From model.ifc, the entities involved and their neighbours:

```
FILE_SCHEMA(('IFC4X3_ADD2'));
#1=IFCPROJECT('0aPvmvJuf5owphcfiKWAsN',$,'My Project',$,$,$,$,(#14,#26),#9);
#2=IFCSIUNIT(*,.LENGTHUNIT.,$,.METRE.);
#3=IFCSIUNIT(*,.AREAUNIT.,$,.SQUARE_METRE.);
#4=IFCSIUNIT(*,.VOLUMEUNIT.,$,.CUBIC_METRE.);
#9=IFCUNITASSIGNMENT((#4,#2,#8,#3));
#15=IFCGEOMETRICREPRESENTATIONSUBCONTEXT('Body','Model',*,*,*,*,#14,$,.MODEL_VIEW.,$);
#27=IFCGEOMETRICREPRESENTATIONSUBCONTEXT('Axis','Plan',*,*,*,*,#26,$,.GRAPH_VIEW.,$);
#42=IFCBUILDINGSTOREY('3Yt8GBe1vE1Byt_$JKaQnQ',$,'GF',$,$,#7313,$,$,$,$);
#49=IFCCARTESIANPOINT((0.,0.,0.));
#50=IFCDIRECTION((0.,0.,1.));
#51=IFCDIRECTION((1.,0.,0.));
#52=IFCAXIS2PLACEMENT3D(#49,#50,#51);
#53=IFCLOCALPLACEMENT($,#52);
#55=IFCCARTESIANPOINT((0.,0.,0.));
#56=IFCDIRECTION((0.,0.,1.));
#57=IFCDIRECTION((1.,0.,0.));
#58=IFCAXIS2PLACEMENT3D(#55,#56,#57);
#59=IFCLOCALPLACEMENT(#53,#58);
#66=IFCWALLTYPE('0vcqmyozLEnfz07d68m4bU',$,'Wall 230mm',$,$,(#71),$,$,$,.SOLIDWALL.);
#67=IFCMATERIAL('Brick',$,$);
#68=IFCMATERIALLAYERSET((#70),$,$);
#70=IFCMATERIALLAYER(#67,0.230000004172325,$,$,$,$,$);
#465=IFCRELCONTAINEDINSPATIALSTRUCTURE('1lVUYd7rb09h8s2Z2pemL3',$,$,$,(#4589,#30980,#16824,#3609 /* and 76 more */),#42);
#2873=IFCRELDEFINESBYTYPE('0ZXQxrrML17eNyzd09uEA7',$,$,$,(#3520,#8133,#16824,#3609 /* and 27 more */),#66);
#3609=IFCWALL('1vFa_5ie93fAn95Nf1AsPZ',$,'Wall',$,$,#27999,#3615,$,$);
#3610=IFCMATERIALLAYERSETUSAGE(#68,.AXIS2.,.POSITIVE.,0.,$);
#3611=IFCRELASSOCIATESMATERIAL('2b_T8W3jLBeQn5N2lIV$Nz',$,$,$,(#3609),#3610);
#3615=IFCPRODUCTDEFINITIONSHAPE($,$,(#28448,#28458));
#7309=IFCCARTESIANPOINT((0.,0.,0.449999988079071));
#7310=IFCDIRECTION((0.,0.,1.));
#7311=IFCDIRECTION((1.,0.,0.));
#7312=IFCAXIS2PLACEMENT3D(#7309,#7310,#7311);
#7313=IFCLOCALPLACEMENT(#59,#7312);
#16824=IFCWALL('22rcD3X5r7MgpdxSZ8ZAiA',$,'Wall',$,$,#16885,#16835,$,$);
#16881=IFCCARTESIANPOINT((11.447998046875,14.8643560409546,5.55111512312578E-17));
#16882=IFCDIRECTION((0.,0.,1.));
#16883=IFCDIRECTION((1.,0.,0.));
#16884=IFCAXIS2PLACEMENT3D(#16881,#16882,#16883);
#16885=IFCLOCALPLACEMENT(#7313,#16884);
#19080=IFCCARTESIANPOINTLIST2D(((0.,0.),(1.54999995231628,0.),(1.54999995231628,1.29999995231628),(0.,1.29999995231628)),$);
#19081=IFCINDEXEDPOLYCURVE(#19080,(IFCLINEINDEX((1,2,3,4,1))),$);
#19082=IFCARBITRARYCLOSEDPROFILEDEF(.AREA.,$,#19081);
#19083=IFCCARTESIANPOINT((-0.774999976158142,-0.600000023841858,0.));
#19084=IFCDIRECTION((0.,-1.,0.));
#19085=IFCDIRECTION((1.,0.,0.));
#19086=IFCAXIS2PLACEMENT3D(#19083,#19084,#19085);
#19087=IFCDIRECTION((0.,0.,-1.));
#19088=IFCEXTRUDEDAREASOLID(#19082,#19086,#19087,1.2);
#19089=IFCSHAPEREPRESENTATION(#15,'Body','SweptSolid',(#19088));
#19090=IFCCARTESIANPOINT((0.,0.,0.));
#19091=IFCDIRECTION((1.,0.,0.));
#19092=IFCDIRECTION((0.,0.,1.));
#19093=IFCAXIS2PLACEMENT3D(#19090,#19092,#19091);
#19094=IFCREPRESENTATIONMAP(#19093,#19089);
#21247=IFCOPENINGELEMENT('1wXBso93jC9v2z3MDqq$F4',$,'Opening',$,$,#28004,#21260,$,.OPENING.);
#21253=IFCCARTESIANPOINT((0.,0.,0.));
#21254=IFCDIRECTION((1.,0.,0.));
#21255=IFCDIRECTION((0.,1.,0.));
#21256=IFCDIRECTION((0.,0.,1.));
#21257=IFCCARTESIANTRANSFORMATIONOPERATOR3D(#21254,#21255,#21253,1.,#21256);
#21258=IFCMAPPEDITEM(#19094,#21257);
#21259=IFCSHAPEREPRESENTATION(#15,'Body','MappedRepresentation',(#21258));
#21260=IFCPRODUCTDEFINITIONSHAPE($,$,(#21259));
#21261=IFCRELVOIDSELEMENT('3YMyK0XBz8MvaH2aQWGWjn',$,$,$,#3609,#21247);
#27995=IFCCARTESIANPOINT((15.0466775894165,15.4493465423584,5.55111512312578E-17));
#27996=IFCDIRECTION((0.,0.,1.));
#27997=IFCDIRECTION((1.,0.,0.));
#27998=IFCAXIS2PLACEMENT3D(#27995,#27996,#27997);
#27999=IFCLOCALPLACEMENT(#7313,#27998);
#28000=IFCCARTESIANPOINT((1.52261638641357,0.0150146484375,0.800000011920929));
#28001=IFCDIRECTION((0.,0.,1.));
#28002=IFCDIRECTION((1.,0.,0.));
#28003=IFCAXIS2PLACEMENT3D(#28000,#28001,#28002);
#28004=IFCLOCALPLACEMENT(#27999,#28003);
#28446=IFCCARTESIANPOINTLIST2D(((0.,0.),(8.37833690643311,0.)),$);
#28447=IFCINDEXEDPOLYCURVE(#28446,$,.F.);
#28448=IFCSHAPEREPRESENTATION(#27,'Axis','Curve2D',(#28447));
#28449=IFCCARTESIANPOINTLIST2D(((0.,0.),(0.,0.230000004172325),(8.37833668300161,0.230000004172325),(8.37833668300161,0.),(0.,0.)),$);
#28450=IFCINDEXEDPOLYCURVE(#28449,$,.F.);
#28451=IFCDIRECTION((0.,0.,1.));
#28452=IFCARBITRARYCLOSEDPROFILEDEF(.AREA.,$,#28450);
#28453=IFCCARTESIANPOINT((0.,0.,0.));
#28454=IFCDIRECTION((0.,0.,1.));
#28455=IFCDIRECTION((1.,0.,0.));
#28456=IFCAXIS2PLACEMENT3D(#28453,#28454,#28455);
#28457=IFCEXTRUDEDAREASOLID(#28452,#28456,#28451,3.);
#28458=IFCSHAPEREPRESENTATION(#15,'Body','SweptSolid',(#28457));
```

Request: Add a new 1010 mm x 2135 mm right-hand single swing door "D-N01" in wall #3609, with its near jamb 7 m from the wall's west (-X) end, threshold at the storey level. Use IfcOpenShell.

```python
import numpy as np
import ifcopenshell
import ifcopenshell.api.feature
import ifcopenshell.api.geometry
import ifcopenshell.api.root
import ifcopenshell.api.spatial
import ifcopenshell.geom
import ifcopenshell.util.element
import ifcopenshell.util.placement
import ifcopenshell.util.representation
import ifcopenshell.util.shape
import ifcopenshell.util.unit

model = ifcopenshell.open("model.ifc")
unit_scale = ifcopenshell.util.unit.calculate_unit_scale(model)
settings = ifcopenshell.geom.settings()


def volume(element):
    """Net volume in cubic metres, openings subtracted."""
    shape = ifcopenshell.geom.create_shape(settings, element)
    return ifcopenshell.util.shape.get_volume(shape.geometry)


wall = model.by_guid("1vFa_5ie93fAn95Nf1AsPZ")
storey = ifcopenshell.util.element.get_container(wall, ifc_class="IfcBuildingStorey")
context = ifcopenshell.util.representation.get_context(model, "Model", "Body", "MODEL_VIEW")
before = volume(wall)

width, height, from_end, sill = 1.01, 2.135, 7, 0.0  # metres

# The wall runs along its own X axis, and the end named is its -X end.
wall_shape = ifcopenshell.geom.create_shape(settings, wall)
x, y, z = ifcopenshell.util.shape.get_vertices(wall_shape.geometry).T
start = x.min() + from_end
face, thickness = float(y.min()), float(y.max() - y.min())
wall_matrix = ifcopenshell.util.placement.get_local_placement(wall.ObjectPlacement)
level = ifcopenshell.util.placement.get_local_placement(storey.ObjectPlacement)[2, 3]


def in_wall(x, y):
    """Placement at x, y metres in the wall's axes, at sill height."""
    matrix = wall_matrix.copy()
    matrix[:, 3] = wall_matrix @ np.array([x / unit_scale, y / unit_scale, 0.0, 1.0])
    matrix[2, 3] = level + sill / unit_scale
    return matrix


# Opening: a box that overshoots both wall faces by 50 mm.
opening = ifcopenshell.api.root.create_entity(model, ifc_class="IfcOpeningElement", predefined_type="OPENING")
box = ifcopenshell.api.geometry.add_wall_representation(
    model, context=context, length=width, height=height, thickness=thickness + 0.1
)
ifcopenshell.api.geometry.assign_representation(model, product=opening, representation=box)
ifcopenshell.api.geometry.edit_object_placement(model, product=opening, matrix=in_wall(start, face - 0.05), is_si=False)
ifcopenshell.api.feature.add_feature(model, feature=opening, element=wall)

door = ifcopenshell.api.root.create_entity(model, ifc_class="IfcDoor", name="D-N01", predefined_type="DOOR")
door.OverallWidth, door.OverallHeight = width / unit_scale, height / unit_scale
door.OperationType = "SINGLE_SWING_RIGHT"
body = ifcopenshell.api.geometry.add_door_representation(
    model,
    context=context,
    overall_width=door.OverallWidth,
    overall_height=door.OverallHeight,
    operation_type="SINGLE_SWING_RIGHT",
    lining_properties={"LiningDepth": thickness / unit_scale, "ThresholdDepth": thickness / unit_scale},
)
ifcopenshell.api.geometry.assign_representation(model, product=door, representation=body)
ifcopenshell.api.spatial.assign_container(model, products=[door], relating_structure=storey)
ifcopenshell.api.feature.add_filling(model, opening=opening, element=door)

# The lining spans the wall, so the door starts at the wall face.
ifcopenshell.api.geometry.edit_object_placement(model, product=door, matrix=in_wall(start, face), is_si=False)

after = volume(wall)

print(f"wall volume {before:.3f} -> {after:.3f} m3")

model.write("model_rev.ifc")
```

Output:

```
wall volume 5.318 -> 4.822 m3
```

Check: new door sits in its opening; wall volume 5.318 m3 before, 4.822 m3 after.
